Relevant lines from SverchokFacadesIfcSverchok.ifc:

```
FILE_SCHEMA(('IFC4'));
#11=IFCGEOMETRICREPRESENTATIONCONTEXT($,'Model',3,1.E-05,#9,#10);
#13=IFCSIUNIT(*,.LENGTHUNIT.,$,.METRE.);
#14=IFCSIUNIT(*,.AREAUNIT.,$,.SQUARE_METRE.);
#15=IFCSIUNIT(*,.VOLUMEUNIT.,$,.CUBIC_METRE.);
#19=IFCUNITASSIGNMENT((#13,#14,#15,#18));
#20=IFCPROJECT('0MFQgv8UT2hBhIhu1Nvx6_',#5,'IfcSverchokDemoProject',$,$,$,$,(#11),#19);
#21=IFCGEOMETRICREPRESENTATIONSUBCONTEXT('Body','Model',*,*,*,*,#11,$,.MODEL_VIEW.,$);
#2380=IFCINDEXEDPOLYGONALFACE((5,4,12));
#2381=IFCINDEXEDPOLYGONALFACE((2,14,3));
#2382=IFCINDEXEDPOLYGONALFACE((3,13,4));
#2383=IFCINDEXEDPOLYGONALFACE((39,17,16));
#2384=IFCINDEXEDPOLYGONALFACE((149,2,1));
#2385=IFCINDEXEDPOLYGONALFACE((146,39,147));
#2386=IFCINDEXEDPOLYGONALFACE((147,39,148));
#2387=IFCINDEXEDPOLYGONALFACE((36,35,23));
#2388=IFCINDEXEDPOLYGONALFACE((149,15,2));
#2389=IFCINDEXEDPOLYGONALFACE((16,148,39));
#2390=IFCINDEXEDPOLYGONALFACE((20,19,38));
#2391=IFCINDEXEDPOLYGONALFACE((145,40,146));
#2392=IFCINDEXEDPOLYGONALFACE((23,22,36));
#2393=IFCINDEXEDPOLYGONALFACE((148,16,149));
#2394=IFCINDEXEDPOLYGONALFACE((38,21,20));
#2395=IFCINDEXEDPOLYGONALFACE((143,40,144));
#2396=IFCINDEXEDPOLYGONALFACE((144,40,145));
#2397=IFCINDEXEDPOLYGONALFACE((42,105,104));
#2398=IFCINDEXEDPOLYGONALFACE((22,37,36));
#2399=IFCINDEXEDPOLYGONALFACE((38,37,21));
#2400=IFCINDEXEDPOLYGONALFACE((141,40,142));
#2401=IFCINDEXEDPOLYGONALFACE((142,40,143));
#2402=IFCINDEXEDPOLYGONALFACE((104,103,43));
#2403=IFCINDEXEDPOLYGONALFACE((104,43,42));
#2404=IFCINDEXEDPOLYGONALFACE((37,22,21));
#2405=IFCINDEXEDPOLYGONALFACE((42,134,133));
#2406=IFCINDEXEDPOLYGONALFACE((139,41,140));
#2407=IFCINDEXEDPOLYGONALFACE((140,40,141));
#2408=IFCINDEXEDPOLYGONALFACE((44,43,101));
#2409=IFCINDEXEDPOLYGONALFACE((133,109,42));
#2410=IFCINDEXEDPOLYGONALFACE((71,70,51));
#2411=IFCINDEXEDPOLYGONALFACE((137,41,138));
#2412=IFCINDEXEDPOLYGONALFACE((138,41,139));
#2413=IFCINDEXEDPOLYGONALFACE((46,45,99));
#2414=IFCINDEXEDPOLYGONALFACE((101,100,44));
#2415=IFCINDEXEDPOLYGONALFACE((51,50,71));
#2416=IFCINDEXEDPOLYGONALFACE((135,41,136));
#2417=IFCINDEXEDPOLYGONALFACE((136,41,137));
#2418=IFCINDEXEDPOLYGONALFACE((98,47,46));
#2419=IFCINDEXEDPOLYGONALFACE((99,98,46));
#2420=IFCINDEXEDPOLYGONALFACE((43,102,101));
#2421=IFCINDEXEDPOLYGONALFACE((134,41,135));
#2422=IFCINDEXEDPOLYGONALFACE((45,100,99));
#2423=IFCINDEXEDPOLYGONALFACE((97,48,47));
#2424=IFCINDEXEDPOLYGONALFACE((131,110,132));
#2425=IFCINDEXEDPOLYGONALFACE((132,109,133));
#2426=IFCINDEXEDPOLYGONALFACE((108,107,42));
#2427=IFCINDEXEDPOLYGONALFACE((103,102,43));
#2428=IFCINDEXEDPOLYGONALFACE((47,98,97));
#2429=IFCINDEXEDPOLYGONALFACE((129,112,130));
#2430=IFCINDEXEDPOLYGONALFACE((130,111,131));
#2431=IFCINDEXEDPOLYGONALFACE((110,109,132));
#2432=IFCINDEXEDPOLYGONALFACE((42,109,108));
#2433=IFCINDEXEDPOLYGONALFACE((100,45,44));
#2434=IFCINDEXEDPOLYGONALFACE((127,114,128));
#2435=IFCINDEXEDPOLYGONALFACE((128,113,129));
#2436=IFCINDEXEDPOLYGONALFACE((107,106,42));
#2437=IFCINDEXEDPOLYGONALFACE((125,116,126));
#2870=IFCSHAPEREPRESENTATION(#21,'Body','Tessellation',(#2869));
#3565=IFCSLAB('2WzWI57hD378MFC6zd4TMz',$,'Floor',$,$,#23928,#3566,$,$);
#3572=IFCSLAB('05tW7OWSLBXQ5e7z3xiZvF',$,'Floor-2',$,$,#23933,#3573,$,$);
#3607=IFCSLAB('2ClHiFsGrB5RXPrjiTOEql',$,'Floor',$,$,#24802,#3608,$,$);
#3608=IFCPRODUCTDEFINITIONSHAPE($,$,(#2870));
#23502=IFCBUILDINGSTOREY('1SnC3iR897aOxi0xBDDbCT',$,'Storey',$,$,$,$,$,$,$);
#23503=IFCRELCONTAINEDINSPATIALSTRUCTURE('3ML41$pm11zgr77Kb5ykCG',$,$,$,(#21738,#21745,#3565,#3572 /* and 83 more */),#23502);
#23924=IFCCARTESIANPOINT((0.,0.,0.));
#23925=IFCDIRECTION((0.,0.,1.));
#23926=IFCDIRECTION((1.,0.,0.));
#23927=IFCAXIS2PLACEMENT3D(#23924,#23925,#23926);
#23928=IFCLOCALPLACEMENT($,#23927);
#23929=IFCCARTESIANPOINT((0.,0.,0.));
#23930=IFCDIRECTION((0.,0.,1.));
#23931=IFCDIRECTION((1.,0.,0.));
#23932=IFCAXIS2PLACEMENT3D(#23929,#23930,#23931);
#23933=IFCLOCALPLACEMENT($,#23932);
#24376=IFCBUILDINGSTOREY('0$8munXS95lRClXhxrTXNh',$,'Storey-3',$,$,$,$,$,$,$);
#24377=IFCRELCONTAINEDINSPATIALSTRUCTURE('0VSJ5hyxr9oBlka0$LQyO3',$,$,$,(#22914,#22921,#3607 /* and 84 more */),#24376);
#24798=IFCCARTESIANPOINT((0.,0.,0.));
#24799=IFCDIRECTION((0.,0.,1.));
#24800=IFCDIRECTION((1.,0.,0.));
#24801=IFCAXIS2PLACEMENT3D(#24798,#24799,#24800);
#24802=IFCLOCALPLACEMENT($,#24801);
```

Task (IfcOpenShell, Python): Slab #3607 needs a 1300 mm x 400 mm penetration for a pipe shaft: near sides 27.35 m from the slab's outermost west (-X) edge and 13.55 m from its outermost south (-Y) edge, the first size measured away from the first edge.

```python
import numpy as np
import ifcopenshell
import ifcopenshell.api.feature
import ifcopenshell.api.geometry
import ifcopenshell.api.root
import ifcopenshell.geom
import ifcopenshell.util.placement
import ifcopenshell.util.representation
import ifcopenshell.util.shape
import ifcopenshell.util.unit

model = ifcopenshell.open("SverchokFacadesIfcSverchok.ifc")
unit_scale = ifcopenshell.util.unit.calculate_unit_scale(model)
settings = ifcopenshell.geom.settings()


def volume(element):
    """Net volume in cubic metres, openings subtracted."""
    shape = ifcopenshell.geom.create_shape(settings, element)
    return ifcopenshell.util.shape.get_volume(shape.geometry)


slab = model.by_guid("2ClHiFsGrB5RXPrjiTOEql")
before = volume(slab)

# Extent in the slab's own axes, in metres. The edges named are its -X and -Y sides.
slab_shape = ifcopenshell.geom.create_shape(settings, slab)
vertices = ifcopenshell.util.shape.get_vertices(slab_shape.geometry)
x_min, y_min, bottom = vertices.min(axis=0)
top = vertices[:, 2].max()

opening = ifcopenshell.api.root.create_entity(model, ifc_class="IfcOpeningElement", name="Pipe shaft opening", predefined_type="OPENING")
context = ifcopenshell.util.representation.get_context(model, "Model", "Body", "MODEL_VIEW")
width, depth = 1.3, 0.4
outline = [(0.0, 0.0), (width, 0.0), (width, depth), (0.0, depth), (0.0, 0.0)]
# Overshoot both faces by 50 mm so the cut is clean.
shape = ifcopenshell.api.geometry.add_slab_representation(
    model, context=context, depth=top - bottom + 0.1, polyline=outline
)
ifcopenshell.api.geometry.assign_representation(model, product=opening, representation=shape)

matrix = ifcopenshell.util.placement.get_local_placement(slab.ObjectPlacement)
matrix[:, 3] = matrix @ np.append(np.array([x_min + 27.35, y_min + 13.55, bottom - 0.05]) / unit_scale, 1.0)
ifcopenshell.api.geometry.edit_object_placement(model, product=opening, matrix=matrix, is_si=False)
ifcopenshell.api.feature.add_feature(model, feature=opening, element=slab)

after = volume(slab)

print(f"slab volume {before:.3f} -> {after:.3f} m3")

model.write("SverchokFacadesIfcSverchok_edited.ifc")
```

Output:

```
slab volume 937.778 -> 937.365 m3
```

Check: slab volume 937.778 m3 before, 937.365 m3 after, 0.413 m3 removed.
